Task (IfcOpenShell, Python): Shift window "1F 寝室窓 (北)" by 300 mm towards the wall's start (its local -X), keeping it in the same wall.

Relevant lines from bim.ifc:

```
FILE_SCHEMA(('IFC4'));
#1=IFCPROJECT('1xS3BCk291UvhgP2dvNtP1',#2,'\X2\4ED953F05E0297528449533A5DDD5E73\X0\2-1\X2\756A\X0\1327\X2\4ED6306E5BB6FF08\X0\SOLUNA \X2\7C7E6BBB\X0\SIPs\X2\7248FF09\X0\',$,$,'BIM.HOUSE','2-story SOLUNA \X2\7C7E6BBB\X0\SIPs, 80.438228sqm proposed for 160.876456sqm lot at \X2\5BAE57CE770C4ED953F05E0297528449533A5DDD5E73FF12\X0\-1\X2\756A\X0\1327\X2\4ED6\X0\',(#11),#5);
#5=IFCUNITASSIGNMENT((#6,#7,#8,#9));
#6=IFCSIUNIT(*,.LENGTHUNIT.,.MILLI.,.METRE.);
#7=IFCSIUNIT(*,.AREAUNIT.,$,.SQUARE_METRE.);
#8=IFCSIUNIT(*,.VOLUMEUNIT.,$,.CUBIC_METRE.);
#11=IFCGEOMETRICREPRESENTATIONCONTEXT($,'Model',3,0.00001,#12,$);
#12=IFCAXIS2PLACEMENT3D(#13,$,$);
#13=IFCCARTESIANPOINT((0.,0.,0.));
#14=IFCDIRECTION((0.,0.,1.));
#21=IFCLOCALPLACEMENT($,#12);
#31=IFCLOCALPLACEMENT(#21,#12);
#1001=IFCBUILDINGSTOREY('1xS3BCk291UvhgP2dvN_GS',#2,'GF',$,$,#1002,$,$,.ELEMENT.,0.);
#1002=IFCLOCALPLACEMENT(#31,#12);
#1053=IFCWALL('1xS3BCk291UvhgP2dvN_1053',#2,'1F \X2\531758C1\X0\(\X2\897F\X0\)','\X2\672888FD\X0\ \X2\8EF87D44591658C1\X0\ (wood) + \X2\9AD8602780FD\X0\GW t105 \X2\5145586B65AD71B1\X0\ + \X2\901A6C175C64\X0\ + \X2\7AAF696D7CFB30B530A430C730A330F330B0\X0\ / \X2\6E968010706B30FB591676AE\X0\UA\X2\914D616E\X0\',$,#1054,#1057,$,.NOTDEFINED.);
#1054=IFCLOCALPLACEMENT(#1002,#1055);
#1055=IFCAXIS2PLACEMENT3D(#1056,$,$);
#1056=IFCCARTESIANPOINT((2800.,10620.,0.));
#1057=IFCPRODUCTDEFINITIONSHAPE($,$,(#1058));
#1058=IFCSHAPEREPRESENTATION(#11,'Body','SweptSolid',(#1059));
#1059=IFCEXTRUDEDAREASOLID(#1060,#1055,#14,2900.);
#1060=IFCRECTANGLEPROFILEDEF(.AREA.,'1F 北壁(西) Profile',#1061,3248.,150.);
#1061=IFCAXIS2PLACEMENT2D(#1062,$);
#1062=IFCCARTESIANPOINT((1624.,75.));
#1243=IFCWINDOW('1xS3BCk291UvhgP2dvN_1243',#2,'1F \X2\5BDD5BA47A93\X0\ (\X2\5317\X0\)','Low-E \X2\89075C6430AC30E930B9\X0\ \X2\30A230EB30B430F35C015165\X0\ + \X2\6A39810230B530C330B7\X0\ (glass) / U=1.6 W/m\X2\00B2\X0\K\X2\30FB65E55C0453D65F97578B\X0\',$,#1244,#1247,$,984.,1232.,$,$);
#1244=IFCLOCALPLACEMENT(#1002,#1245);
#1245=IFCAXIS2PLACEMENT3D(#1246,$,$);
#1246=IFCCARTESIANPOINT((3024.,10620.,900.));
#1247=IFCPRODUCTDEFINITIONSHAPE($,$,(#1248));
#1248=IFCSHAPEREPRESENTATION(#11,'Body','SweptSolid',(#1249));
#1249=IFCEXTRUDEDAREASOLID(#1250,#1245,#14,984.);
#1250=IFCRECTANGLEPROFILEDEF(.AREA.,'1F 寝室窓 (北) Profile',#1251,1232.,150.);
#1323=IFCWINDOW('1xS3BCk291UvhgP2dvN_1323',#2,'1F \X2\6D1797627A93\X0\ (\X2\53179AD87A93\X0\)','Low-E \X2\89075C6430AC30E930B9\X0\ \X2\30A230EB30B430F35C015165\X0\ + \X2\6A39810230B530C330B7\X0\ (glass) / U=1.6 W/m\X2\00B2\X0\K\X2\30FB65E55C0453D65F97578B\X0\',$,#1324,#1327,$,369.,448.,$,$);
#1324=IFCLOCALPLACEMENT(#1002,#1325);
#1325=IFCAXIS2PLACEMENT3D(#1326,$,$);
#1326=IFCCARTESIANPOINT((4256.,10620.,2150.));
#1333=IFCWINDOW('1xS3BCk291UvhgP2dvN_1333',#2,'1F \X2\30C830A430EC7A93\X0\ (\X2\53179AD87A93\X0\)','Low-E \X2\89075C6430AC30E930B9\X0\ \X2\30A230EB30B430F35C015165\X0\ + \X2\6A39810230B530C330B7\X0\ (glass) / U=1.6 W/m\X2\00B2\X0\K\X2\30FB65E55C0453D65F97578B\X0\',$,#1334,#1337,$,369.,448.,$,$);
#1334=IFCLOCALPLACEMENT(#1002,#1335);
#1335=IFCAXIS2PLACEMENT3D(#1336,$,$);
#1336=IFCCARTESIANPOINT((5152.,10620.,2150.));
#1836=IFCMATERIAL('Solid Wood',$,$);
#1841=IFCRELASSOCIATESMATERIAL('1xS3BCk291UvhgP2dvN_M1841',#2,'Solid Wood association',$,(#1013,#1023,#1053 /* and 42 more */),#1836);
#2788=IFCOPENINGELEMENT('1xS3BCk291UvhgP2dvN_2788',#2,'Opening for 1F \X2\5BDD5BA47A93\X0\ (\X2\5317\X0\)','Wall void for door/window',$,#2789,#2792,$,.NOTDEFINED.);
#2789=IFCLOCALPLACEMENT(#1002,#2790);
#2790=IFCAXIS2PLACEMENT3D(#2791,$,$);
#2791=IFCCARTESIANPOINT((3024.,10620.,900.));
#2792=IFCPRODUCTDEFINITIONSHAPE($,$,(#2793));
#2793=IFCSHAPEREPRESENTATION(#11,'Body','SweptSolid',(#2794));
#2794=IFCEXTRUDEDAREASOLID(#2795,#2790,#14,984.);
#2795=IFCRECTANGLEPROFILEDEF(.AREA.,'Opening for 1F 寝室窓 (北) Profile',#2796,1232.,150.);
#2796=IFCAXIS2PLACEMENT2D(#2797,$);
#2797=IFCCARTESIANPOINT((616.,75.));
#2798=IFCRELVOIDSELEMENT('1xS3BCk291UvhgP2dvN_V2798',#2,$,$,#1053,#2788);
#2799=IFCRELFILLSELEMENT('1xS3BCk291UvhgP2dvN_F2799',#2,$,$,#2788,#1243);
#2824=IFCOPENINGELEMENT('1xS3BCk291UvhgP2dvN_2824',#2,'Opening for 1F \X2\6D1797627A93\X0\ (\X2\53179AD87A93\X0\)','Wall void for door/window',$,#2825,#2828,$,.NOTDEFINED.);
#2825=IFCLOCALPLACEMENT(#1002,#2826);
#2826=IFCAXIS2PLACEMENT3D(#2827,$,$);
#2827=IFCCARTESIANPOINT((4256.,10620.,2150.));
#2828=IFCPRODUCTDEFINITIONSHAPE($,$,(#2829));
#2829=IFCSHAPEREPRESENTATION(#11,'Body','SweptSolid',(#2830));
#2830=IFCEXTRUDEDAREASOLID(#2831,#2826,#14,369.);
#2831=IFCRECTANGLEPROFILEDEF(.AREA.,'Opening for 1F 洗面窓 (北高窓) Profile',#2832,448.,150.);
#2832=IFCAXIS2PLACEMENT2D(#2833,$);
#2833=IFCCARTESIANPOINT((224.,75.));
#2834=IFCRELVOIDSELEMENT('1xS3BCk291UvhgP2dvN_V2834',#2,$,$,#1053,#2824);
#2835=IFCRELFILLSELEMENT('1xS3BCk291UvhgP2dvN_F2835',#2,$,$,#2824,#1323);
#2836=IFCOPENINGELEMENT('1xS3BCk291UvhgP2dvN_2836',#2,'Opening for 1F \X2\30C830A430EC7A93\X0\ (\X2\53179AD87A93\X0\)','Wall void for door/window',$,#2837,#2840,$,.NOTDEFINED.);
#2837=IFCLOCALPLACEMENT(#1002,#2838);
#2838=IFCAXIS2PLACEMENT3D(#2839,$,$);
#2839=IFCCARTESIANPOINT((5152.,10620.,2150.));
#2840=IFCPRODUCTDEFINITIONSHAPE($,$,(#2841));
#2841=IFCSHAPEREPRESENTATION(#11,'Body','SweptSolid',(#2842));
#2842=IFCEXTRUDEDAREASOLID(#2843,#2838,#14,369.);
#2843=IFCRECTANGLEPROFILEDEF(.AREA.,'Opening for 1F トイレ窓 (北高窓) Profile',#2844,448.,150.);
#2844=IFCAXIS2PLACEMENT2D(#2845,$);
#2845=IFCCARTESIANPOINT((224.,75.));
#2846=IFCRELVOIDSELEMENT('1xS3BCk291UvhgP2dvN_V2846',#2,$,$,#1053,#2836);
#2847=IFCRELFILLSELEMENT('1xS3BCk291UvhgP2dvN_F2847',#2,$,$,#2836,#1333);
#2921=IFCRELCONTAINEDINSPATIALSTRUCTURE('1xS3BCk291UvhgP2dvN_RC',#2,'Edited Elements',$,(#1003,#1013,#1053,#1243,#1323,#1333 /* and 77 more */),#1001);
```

```python
import ifcopenshell
import ifcopenshell.api.geometry
import ifcopenshell.util.placement

model = ifcopenshell.open("bim.ifc")

window = model.by_id(1243)
opening = window.FillsVoids[0].RelatingOpeningElement
wall = opening.VoidsElements[0].RelatingBuildingElement

wall_matrix = ifcopenshell.util.placement.get_local_placement(wall.ObjectPlacement)
shift = wall_matrix[:3, 0] * -300.0
before = ifcopenshell.util.placement.get_local_placement(window.ObjectPlacement)[:3, 3].copy()

# The window is not placed relative to its opening, so move both.
for product in (opening, window):
    matrix = ifcopenshell.util.placement.get_local_placement(product.ObjectPlacement)
    matrix[:3, 3] += shift
    ifcopenshell.api.geometry.edit_object_placement(model, product=product, matrix=matrix, is_si=False)

after = ifcopenshell.util.placement.get_local_placement(window.ObjectPlacement)[:3, 3]
print("window moved by", (after - before).round(3) + 0.0)

model.write("bim_edited.ifc")
```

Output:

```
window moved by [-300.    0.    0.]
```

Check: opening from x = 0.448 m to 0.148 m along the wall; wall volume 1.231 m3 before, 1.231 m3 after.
